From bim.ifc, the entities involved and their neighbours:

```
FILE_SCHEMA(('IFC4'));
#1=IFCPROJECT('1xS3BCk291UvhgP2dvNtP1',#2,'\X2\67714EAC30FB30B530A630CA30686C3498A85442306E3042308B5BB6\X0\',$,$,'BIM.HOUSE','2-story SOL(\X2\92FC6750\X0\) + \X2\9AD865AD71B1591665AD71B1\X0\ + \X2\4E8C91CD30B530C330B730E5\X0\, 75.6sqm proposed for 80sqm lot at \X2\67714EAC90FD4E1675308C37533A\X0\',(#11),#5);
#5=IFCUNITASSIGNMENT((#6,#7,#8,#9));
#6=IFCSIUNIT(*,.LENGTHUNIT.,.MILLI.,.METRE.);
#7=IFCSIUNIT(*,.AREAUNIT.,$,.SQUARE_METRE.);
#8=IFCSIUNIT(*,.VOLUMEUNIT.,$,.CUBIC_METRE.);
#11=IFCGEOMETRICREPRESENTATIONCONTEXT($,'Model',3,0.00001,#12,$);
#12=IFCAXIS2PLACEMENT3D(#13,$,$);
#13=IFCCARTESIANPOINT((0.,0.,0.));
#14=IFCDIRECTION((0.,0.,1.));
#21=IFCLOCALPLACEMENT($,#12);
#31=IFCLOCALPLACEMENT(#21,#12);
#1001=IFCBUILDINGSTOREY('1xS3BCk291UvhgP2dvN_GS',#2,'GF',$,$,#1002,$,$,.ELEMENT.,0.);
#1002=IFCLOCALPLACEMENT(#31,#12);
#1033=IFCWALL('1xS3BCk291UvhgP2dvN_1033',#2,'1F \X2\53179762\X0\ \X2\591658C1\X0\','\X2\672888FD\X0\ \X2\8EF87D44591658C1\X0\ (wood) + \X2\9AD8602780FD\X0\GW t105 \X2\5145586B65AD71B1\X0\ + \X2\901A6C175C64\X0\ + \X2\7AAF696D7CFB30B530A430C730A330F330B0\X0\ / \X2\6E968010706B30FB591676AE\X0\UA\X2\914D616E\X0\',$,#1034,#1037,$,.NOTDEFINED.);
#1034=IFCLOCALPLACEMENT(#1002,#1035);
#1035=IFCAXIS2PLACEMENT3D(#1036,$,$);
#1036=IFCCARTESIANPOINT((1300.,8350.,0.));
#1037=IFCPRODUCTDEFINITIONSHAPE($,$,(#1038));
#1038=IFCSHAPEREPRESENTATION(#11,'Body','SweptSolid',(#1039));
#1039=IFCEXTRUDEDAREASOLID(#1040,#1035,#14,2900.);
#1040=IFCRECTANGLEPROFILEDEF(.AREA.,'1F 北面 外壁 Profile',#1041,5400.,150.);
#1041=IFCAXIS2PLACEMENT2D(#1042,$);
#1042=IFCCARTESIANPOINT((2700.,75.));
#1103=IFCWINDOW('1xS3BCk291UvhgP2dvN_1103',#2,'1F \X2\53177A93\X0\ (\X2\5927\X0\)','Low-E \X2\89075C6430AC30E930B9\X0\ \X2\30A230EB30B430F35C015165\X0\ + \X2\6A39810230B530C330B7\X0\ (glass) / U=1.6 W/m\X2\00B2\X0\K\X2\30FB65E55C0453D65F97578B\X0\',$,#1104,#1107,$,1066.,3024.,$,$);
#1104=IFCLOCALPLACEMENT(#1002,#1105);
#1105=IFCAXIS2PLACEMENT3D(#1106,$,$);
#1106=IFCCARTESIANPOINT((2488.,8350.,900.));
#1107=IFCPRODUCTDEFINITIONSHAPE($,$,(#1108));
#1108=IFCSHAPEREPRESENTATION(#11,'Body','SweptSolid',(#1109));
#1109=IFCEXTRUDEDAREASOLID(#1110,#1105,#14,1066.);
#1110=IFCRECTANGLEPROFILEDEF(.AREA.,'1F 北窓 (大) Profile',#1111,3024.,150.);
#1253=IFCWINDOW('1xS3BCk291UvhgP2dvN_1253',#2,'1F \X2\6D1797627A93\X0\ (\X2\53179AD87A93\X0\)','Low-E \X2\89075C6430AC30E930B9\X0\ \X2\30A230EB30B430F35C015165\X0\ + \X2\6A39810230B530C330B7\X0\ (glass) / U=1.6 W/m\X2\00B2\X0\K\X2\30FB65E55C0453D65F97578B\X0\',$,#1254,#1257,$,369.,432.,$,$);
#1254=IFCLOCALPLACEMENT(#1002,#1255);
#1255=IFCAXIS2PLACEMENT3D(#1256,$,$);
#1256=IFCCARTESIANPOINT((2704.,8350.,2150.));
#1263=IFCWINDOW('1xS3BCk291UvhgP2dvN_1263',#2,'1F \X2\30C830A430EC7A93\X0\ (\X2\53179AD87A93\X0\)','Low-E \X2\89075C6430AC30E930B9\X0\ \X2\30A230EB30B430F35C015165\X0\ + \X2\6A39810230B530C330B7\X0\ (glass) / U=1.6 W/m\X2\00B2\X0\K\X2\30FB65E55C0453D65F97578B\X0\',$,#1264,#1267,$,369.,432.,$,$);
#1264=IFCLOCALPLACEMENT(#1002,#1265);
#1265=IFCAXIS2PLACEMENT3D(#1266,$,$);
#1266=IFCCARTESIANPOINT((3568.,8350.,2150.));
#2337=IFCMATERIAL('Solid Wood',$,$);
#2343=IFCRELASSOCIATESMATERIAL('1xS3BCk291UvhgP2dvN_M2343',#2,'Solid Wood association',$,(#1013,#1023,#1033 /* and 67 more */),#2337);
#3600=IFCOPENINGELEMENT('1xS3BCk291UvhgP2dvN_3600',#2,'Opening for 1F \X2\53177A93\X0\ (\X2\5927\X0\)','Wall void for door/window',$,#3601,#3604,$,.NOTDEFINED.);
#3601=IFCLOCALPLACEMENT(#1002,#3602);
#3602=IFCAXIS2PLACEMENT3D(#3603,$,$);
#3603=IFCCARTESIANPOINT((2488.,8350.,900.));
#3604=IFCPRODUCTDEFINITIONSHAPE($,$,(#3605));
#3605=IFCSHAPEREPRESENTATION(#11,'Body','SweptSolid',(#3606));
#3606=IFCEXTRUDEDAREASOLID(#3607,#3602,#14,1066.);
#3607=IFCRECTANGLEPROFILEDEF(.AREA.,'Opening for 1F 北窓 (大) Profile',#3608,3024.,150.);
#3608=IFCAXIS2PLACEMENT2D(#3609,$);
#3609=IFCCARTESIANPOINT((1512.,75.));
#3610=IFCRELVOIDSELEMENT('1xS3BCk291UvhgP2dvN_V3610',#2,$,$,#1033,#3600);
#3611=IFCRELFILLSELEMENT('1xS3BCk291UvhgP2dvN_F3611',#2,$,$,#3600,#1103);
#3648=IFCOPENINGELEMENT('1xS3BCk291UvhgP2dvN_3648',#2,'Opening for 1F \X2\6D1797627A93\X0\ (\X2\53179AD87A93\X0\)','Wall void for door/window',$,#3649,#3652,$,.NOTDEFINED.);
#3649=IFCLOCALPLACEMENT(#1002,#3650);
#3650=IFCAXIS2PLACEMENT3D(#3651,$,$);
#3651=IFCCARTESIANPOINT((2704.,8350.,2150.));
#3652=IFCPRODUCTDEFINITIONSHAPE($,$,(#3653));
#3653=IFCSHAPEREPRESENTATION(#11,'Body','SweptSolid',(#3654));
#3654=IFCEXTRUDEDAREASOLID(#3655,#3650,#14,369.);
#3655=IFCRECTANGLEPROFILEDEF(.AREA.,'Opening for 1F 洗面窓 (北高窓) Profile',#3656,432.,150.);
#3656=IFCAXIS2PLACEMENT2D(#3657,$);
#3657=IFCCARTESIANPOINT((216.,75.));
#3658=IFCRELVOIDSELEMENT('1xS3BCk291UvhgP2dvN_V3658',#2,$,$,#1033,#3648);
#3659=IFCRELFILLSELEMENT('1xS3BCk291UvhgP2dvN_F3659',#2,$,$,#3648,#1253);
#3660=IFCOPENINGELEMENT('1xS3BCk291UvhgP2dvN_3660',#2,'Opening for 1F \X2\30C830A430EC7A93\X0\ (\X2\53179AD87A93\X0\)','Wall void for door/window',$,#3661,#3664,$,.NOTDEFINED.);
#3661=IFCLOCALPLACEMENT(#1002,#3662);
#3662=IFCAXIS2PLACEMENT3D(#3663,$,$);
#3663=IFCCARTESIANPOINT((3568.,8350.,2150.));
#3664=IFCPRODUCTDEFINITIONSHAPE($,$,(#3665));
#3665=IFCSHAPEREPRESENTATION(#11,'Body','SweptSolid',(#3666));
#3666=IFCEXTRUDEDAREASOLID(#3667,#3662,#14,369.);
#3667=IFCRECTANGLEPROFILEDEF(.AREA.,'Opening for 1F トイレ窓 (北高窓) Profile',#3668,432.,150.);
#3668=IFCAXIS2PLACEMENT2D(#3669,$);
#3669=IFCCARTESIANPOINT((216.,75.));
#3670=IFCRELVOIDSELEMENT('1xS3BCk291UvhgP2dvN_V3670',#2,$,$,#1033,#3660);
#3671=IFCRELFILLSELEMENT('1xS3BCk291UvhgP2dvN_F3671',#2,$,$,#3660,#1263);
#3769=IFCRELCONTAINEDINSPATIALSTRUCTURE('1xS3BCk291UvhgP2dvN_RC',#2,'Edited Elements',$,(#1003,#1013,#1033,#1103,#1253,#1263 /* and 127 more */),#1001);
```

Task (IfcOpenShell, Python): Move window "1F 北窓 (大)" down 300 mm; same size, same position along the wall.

```python
import numpy as np
import ifcopenshell
import ifcopenshell.api.geometry
import ifcopenshell.util.placement
import ifcopenshell.util.unit

model = ifcopenshell.open("bim.ifc")
unit_scale = ifcopenshell.util.unit.calculate_unit_scale(model)

window = model.by_guid("1xS3BCk291UvhgP2dvN_1103")
opening = window.FillsVoids[0].RelatingOpeningElement
dz = -300.0

shift = np.array([0.0, 0.0, dz])
# The window is not placed relative to its opening, so move both.
for product in (opening, window):
    matrix = ifcopenshell.util.placement.get_local_placement(product.ObjectPlacement)
    matrix[:3, 3] += shift
    ifcopenshell.api.geometry.edit_object_placement(model, product=product, matrix=matrix, is_si=False)

print(f"moved by {dz * unit_scale:+.3f} m")

model.write("bim_rev.ifc")
```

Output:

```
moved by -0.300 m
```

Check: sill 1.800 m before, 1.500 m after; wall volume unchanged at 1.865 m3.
